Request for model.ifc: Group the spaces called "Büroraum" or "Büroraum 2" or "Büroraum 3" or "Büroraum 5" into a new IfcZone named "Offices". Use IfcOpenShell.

First a look at what the model holds.

```python
import ifcopenshell

model = ifcopenshell.open("model.ifc")
print(model.schema)
seen = {}
for space in model.by_type("IfcSpace"):
    seen[space.Name] = seen.get(space.Name, 0) + 1
for name, count in sorted(seen.items(), key=str):
    print(count, "x", name)
print("zones:", [z.Name for z in model.by_type("IfcZone")][:20])
```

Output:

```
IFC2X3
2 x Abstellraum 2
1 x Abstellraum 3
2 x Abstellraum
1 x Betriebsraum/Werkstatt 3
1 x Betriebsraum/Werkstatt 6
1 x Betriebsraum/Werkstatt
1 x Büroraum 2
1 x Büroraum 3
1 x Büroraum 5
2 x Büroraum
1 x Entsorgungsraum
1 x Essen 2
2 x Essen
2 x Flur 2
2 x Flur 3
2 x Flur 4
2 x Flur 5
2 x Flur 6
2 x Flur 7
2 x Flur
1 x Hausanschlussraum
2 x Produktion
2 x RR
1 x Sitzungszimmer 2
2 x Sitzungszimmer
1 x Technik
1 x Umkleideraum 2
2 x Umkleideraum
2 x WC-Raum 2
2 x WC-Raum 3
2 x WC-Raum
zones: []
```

```python
import ifcopenshell
import ifcopenshell.api.group
import ifcopenshell.api.root

model = ifcopenshell.open("model.ifc")

names = {"Büroraum", "Büroraum 2", "Büroraum 3", "Büroraum 5"}
spaces = [s for s in model.by_type("IfcSpace") if s.Name in names]

zone = ifcopenshell.api.root.create_entity(model, ifc_class="IfcZone", name="Offices")
ifcopenshell.api.group.assign_group(model, products=spaces, group=zone)
print(len(spaces), "spaces in", zone.Name)

model.write("model_updated.ifc")
```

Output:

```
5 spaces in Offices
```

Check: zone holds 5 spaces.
